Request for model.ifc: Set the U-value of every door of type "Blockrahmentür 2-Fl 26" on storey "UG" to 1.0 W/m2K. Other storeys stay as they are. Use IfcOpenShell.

First a look at what the model holds.

```python
import ifcopenshell
import ifcopenshell.util.element

model = ifcopenshell.open("model.ifc")
print(model.schema)
storey = next(s for s in model.by_type("IfcBuildingStorey") if s.Name == "UG")
doors = [e for e in ifcopenshell.util.element.get_decomposition(storey) if e.is_a("IfcDoor")]
seen = {}
for e in doors:
    element_type = ifcopenshell.util.element.get_type(e)
    key = (element_type.Name if element_type != e and element_type else None, ifcopenshell.util.element.get_pset(e, "Pset_DoorCommon", "ThermalTransmittance"))
    seen[key] = seen.get(key, 0) + 1
for (name, value), count in sorted(seen.items(), key=str):
    print(count, "x", name, "|", value)
```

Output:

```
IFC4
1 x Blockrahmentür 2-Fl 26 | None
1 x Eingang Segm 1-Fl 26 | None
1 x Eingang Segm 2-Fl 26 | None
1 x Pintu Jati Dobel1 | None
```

```python
import ifcopenshell
import ifcopenshell.api.pset
import ifcopenshell.util.element

model = ifcopenshell.open("model.ifc")

storey = next(s for s in model.by_type("IfcBuildingStorey") if s.Name == "UG")
doors = [e for e in ifcopenshell.util.element.get_decomposition(storey) if e.is_a("IfcDoor")]

count = 0
for e in doors:
    element_type = ifcopenshell.util.element.get_type(e)
    if element_type in (None, e) or element_type.Name != "Blockrahmentür 2-Fl 26":
        continue
    # add_pset returns the element's existing set when there is one.
    pset = ifcopenshell.api.pset.add_pset(model, product=e, name="Pset_DoorCommon")
    ifcopenshell.api.pset.edit_pset(model, pset=pset, properties={"ThermalTransmittance": 1.0})
    count += 1

print(count, "doors updated")

model.write("model-out.ifc")
```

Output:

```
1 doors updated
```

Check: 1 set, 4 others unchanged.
